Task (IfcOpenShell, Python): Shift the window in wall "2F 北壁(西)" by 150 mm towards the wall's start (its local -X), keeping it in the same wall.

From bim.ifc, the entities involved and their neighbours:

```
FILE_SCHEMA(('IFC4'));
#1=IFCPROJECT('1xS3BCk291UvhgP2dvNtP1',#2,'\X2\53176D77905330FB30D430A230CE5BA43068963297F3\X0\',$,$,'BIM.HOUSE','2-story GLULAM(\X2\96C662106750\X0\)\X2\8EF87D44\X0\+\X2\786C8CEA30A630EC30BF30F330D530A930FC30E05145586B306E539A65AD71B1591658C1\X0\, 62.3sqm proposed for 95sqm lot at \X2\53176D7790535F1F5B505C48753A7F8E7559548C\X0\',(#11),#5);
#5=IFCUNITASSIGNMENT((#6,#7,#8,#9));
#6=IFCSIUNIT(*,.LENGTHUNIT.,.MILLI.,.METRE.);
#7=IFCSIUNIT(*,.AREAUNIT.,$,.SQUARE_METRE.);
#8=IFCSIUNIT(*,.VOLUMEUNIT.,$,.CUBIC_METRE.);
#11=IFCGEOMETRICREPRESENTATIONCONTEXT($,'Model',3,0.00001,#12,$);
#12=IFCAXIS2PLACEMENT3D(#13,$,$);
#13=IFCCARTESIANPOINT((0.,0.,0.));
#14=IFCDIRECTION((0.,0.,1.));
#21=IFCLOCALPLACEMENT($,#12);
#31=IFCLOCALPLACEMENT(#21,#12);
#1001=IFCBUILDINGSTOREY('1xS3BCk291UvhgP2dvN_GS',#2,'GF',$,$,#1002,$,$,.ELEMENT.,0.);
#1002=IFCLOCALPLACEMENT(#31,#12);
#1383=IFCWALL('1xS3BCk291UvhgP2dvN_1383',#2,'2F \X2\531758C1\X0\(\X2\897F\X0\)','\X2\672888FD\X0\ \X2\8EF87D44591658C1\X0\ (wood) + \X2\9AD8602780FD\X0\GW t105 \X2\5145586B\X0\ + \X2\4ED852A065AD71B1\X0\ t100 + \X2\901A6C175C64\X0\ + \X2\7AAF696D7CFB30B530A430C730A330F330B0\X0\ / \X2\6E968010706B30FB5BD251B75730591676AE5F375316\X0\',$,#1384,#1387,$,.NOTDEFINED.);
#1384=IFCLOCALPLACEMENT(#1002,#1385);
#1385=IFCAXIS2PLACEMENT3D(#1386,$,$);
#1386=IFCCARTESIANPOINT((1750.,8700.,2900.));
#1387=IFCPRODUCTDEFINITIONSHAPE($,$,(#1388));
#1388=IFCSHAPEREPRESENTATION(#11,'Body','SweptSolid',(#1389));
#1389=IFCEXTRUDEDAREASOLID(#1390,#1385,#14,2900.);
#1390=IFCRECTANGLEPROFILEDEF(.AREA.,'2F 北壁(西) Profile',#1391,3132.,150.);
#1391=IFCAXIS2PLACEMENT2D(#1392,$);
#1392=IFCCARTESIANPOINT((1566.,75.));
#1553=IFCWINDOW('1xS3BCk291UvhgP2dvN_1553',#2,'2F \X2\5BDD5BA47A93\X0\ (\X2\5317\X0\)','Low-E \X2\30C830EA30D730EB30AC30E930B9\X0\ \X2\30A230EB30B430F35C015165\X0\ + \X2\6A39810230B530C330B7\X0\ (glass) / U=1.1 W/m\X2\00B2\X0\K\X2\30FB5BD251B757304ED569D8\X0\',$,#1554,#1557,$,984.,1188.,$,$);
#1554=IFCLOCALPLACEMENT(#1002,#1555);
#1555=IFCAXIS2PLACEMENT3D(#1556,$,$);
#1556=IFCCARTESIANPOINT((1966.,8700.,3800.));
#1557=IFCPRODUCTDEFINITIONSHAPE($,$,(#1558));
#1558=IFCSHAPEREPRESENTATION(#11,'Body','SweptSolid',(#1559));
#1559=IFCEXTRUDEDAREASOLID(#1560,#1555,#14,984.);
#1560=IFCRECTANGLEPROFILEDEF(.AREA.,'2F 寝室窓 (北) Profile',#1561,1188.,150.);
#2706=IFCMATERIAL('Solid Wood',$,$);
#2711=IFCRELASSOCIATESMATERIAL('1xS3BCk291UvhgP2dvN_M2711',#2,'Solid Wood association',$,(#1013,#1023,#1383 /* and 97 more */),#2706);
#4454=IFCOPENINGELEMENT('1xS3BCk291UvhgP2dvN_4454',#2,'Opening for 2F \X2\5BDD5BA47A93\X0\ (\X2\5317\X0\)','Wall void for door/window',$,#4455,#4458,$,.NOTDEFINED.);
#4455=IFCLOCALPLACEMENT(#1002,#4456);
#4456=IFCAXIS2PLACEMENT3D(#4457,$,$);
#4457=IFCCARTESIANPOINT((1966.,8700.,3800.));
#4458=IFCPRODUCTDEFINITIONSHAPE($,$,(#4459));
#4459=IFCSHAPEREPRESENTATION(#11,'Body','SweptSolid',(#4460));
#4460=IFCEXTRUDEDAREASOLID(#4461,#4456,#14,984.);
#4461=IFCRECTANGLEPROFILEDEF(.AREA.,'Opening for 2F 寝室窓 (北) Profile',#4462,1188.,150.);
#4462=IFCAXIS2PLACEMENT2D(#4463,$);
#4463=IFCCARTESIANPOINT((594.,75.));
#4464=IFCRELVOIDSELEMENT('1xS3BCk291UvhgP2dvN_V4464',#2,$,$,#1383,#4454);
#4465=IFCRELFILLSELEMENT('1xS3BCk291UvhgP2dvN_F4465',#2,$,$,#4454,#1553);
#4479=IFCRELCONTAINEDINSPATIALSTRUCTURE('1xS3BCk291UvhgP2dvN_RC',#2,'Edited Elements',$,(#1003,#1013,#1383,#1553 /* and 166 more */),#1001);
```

```python
import ifcopenshell
import ifcopenshell.api.geometry
import ifcopenshell.util.placement
import ifcopenshell.util.unit

model = ifcopenshell.open("bim.ifc")
unit_scale = ifcopenshell.util.unit.calculate_unit_scale(model)

window = model.by_guid("1xS3BCk291UvhgP2dvN_1553")
opening = window.FillsVoids[0].RelatingOpeningElement
wall = opening.VoidsElements[0].RelatingBuildingElement

wall_matrix = ifcopenshell.util.placement.get_local_placement(wall.ObjectPlacement)
shift = wall_matrix[:3, 0] * -0.15 / unit_scale
before = ifcopenshell.util.placement.get_local_placement(window.ObjectPlacement)[:3, 3].copy()

# The window is not placed relative to its opening, so move both.
for product in (opening, window):
    matrix = ifcopenshell.util.placement.get_local_placement(product.ObjectPlacement)
    matrix[:3, 3] += shift
    ifcopenshell.api.geometry.edit_object_placement(model, product=product, matrix=matrix, is_si=False)

after = ifcopenshell.util.placement.get_local_placement(window.ObjectPlacement)[:3, 3]
print("window moved by", (after - before).round(3) + 0.0)

model.write("bim_rev.ifc")
```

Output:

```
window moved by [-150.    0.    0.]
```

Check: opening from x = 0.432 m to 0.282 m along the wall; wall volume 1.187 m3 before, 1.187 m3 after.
